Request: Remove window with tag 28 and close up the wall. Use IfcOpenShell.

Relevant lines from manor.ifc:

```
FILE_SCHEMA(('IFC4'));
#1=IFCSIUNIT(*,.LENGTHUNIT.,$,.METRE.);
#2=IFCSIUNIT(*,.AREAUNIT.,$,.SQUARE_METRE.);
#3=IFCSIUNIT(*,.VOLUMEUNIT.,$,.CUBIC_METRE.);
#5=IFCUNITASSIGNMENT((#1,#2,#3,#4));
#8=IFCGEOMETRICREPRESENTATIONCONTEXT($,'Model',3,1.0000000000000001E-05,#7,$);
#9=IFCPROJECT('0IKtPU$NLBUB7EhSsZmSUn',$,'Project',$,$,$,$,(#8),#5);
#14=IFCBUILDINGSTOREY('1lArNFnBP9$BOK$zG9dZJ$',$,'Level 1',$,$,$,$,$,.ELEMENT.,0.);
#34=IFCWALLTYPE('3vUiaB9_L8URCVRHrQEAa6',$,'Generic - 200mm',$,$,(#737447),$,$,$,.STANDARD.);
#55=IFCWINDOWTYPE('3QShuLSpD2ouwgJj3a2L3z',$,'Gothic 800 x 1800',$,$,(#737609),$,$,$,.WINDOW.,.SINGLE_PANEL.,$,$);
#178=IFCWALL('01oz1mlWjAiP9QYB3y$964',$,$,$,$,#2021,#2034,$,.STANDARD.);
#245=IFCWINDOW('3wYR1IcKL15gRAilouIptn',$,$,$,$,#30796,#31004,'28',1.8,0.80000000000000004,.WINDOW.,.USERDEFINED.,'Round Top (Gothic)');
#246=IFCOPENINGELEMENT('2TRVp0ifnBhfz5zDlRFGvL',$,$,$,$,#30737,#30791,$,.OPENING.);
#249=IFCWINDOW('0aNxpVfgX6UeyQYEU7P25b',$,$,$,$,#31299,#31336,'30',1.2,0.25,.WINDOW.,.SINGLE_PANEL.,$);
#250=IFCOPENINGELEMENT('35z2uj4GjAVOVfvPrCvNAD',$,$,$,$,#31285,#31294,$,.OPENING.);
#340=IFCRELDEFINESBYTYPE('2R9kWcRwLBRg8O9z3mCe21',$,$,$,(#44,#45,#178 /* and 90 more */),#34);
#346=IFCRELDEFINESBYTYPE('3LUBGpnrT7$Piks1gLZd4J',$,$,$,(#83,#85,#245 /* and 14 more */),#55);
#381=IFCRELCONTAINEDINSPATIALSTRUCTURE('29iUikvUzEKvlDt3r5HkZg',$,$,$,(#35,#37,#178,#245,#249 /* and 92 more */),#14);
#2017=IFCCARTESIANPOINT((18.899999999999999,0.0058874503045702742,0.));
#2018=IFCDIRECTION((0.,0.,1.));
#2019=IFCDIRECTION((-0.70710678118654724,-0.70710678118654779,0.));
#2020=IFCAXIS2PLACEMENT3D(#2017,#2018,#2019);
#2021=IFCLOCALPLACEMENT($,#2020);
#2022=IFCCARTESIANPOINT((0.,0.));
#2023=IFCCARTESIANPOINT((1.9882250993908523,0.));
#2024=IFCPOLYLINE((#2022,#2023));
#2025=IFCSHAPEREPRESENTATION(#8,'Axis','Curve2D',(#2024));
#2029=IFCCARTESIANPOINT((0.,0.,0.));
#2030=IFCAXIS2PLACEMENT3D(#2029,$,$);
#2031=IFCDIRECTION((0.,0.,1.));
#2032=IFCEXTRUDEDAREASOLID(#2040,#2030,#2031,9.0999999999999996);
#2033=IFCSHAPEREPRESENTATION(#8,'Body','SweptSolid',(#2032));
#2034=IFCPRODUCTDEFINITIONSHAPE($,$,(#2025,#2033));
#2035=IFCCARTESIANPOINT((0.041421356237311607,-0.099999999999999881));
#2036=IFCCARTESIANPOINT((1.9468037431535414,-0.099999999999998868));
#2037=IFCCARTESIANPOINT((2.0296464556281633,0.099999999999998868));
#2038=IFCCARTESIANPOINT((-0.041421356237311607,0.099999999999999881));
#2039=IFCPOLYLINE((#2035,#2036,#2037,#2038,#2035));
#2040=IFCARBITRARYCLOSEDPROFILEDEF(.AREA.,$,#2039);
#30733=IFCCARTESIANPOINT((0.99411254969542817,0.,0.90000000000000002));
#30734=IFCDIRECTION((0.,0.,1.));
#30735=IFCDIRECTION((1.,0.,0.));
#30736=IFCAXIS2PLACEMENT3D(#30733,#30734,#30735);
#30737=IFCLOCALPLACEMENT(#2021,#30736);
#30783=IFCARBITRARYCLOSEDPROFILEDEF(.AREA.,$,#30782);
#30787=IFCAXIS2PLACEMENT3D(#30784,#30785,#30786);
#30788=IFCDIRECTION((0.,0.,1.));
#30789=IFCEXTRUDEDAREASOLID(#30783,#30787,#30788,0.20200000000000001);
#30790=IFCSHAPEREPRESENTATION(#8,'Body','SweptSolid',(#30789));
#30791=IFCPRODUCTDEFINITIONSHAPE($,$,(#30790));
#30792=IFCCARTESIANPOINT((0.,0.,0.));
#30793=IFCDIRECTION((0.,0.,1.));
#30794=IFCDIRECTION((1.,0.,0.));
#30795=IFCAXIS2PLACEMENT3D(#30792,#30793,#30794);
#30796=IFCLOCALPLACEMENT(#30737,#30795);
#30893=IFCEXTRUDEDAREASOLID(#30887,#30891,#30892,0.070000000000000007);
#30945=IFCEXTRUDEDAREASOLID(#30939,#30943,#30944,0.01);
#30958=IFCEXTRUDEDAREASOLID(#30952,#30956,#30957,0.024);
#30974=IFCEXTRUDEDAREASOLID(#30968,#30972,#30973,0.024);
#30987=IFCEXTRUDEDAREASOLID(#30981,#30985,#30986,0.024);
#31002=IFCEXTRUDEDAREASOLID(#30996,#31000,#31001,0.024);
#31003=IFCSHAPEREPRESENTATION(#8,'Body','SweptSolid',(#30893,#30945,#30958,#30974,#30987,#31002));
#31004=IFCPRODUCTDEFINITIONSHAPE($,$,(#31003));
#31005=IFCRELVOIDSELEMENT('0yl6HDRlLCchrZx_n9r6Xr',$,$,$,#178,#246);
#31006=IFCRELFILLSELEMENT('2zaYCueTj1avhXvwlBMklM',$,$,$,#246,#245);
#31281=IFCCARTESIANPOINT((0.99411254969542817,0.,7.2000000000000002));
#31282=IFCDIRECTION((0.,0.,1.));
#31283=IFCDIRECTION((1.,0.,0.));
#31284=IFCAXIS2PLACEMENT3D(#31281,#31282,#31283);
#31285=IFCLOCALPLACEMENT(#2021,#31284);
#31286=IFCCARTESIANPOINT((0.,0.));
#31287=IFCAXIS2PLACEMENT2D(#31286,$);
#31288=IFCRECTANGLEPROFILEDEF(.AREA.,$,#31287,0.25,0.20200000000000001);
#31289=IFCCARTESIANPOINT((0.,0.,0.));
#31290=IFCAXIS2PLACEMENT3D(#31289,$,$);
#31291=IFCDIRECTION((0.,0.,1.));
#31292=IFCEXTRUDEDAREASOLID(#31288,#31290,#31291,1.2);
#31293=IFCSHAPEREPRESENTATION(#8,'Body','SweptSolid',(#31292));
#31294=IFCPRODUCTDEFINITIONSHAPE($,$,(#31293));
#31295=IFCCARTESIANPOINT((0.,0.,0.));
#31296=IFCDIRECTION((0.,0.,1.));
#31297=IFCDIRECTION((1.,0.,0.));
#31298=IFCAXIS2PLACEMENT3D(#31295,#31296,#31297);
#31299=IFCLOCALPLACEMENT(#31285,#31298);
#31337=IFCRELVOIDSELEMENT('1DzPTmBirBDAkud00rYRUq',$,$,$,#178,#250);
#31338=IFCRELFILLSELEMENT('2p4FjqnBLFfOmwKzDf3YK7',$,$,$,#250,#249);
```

```python
import ifcopenshell
import ifcopenshell.api.feature
import ifcopenshell.api.root
import ifcopenshell.geom
import ifcopenshell.util.shape

model = ifcopenshell.open("manor.ifc")
settings = ifcopenshell.geom.settings()


def volume(element):
    """Net volume in cubic metres, openings subtracted."""
    shape = ifcopenshell.geom.create_shape(settings, element)
    return ifcopenshell.util.shape.get_volume(shape.geometry)


window = model.by_guid("3wYR1IcKL15gRAilouIptn")
opening = window.FillsVoids[0].RelatingOpeningElement
wall = opening.VoidsElements[0].RelatingBuildingElement
before = volume(wall)

ifcopenshell.api.root.remove_product(model, product=window)
ifcopenshell.api.feature.remove_feature(model, feature=opening)

after = volume(wall)

print(f"wall volume {before:.3f} -> {after:.3f} m3")

model.write("manor_rev.ifc")
```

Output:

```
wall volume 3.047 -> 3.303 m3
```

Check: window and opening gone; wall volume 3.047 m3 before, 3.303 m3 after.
